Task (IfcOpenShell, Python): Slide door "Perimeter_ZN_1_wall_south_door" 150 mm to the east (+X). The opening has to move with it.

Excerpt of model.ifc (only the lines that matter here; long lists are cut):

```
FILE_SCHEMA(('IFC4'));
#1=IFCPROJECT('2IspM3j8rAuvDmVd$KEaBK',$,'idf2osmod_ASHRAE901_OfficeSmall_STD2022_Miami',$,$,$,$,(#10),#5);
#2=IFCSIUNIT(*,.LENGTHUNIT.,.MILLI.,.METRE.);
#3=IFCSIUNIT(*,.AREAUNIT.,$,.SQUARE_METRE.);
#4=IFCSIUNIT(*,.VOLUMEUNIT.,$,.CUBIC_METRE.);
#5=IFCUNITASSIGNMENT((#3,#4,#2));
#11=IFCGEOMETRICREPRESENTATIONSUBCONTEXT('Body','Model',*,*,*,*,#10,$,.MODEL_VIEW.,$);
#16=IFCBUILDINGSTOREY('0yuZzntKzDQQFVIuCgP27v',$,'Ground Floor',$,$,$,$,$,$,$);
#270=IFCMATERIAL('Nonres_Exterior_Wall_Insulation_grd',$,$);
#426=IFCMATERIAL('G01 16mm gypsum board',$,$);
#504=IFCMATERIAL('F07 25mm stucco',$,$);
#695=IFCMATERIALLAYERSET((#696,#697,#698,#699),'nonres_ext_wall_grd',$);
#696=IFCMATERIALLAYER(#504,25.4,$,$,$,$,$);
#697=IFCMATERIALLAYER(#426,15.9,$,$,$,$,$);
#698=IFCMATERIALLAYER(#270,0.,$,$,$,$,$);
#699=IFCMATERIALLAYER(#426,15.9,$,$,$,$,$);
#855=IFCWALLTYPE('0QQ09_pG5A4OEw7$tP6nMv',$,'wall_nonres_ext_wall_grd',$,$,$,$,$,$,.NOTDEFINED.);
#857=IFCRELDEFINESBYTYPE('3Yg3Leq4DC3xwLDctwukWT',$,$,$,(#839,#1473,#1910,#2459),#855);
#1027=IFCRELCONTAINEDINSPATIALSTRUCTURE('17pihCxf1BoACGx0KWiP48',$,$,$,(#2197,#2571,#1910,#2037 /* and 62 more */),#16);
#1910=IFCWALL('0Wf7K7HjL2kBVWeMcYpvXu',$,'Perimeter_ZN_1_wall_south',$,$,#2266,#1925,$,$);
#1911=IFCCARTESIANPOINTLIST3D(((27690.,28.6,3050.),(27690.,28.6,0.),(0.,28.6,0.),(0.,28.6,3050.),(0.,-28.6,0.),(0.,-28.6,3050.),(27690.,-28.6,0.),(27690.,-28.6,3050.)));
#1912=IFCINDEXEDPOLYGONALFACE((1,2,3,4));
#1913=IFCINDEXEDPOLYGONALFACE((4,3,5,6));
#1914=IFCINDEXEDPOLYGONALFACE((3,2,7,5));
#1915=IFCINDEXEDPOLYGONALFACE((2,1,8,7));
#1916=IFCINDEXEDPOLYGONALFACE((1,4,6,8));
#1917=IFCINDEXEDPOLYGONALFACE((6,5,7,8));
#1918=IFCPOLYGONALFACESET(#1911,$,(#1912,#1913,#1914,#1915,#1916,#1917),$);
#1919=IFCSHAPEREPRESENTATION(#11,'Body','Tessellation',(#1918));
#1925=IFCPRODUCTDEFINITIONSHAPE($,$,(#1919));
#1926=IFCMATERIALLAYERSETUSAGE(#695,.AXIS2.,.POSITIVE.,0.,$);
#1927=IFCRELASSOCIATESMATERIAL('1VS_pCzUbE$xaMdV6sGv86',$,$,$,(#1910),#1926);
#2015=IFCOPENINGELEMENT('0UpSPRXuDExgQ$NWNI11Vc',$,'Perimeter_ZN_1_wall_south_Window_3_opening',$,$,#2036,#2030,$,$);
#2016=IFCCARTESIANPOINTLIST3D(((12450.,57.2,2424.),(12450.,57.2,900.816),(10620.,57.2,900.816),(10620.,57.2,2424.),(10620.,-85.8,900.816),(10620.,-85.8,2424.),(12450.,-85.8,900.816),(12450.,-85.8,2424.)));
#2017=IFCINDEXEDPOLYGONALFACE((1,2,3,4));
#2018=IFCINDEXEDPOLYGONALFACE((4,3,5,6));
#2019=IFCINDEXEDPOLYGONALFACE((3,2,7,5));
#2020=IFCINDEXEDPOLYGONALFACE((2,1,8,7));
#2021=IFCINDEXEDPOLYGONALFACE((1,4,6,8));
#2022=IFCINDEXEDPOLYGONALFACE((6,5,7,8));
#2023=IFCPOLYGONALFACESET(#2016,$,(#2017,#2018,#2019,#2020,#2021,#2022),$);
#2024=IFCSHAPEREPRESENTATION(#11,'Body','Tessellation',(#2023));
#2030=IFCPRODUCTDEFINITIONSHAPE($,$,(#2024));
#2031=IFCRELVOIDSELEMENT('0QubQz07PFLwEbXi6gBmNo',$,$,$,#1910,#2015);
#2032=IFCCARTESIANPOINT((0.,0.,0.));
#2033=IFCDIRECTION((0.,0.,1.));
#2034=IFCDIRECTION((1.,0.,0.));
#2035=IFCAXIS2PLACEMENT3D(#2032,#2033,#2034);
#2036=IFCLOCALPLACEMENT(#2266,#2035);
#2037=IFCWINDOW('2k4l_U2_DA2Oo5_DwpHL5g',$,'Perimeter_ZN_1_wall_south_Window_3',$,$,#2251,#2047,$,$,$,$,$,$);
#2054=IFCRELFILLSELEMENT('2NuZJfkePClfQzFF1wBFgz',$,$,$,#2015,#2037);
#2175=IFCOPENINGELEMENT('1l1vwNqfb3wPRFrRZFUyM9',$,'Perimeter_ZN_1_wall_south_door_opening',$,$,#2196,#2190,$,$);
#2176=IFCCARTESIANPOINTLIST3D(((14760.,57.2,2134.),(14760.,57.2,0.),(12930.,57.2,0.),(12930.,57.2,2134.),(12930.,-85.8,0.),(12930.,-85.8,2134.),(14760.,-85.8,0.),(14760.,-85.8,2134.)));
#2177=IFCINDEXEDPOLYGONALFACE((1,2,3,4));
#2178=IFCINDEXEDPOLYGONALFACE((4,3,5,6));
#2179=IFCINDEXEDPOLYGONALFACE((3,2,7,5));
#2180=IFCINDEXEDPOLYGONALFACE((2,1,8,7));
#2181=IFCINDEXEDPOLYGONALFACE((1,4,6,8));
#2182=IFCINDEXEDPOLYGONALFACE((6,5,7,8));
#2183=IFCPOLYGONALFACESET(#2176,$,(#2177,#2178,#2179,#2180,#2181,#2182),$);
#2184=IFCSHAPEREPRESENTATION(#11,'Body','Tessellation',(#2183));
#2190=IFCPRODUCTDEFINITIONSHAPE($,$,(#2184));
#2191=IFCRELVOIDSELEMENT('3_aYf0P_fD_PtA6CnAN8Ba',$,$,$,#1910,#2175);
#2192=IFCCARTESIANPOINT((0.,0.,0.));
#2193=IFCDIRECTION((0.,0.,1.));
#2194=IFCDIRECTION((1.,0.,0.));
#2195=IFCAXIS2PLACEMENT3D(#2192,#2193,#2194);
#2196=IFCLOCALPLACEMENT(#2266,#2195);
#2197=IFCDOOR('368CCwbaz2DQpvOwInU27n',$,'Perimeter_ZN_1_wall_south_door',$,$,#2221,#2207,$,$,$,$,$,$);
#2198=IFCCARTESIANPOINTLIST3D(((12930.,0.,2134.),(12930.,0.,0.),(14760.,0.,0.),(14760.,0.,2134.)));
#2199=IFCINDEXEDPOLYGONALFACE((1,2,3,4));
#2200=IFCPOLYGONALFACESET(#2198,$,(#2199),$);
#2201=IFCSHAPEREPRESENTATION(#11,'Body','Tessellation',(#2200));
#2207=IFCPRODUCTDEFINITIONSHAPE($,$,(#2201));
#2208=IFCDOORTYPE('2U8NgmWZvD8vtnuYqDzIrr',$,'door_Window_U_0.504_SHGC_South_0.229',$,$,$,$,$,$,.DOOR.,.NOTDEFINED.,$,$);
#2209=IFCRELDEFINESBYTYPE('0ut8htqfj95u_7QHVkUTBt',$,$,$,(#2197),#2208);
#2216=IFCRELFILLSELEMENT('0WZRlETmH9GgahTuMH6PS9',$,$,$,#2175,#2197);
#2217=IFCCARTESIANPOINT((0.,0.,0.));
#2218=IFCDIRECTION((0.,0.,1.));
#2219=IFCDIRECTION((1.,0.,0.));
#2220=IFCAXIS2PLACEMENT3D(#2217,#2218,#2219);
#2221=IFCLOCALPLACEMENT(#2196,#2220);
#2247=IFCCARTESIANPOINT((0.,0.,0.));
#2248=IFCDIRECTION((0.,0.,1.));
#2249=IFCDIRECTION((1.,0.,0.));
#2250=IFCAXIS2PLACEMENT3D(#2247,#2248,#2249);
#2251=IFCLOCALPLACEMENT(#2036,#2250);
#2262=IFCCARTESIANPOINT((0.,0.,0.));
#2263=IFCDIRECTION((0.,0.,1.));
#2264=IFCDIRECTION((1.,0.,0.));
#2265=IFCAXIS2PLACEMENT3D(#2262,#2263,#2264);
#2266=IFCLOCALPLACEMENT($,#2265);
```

```python
import ifcopenshell
import ifcopenshell.api.geometry
import ifcopenshell.util.placement
import ifcopenshell.util.unit

model = ifcopenshell.open("model.ifc")
unit_scale = ifcopenshell.util.unit.calculate_unit_scale(model)

door = model.by_id(2197)
opening = door.FillsVoids[0].RelatingOpeningElement
wall = opening.VoidsElements[0].RelatingBuildingElement

wall_matrix = ifcopenshell.util.placement.get_local_placement(wall.ObjectPlacement)
shift = wall_matrix[:3, 0] * 0.15 / unit_scale
before = ifcopenshell.util.placement.get_local_placement(door.ObjectPlacement)[:3, 3].copy()

# The door is placed relative to its opening, so it follows when the opening moves.
matrix = ifcopenshell.util.placement.get_local_placement(opening.ObjectPlacement)
matrix[:3, 3] += shift
ifcopenshell.api.geometry.edit_object_placement(
    model, product=opening, matrix=matrix, is_si=False, should_transform_children=True
)

after = ifcopenshell.util.placement.get_local_placement(door.ObjectPlacement)[:3, 3]
print("door moved by", (after - before).round(3) + 0.0)

model.write("model_edited.ifc")
```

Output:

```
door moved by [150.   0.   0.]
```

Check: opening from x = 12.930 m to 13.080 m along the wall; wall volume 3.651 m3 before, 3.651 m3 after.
